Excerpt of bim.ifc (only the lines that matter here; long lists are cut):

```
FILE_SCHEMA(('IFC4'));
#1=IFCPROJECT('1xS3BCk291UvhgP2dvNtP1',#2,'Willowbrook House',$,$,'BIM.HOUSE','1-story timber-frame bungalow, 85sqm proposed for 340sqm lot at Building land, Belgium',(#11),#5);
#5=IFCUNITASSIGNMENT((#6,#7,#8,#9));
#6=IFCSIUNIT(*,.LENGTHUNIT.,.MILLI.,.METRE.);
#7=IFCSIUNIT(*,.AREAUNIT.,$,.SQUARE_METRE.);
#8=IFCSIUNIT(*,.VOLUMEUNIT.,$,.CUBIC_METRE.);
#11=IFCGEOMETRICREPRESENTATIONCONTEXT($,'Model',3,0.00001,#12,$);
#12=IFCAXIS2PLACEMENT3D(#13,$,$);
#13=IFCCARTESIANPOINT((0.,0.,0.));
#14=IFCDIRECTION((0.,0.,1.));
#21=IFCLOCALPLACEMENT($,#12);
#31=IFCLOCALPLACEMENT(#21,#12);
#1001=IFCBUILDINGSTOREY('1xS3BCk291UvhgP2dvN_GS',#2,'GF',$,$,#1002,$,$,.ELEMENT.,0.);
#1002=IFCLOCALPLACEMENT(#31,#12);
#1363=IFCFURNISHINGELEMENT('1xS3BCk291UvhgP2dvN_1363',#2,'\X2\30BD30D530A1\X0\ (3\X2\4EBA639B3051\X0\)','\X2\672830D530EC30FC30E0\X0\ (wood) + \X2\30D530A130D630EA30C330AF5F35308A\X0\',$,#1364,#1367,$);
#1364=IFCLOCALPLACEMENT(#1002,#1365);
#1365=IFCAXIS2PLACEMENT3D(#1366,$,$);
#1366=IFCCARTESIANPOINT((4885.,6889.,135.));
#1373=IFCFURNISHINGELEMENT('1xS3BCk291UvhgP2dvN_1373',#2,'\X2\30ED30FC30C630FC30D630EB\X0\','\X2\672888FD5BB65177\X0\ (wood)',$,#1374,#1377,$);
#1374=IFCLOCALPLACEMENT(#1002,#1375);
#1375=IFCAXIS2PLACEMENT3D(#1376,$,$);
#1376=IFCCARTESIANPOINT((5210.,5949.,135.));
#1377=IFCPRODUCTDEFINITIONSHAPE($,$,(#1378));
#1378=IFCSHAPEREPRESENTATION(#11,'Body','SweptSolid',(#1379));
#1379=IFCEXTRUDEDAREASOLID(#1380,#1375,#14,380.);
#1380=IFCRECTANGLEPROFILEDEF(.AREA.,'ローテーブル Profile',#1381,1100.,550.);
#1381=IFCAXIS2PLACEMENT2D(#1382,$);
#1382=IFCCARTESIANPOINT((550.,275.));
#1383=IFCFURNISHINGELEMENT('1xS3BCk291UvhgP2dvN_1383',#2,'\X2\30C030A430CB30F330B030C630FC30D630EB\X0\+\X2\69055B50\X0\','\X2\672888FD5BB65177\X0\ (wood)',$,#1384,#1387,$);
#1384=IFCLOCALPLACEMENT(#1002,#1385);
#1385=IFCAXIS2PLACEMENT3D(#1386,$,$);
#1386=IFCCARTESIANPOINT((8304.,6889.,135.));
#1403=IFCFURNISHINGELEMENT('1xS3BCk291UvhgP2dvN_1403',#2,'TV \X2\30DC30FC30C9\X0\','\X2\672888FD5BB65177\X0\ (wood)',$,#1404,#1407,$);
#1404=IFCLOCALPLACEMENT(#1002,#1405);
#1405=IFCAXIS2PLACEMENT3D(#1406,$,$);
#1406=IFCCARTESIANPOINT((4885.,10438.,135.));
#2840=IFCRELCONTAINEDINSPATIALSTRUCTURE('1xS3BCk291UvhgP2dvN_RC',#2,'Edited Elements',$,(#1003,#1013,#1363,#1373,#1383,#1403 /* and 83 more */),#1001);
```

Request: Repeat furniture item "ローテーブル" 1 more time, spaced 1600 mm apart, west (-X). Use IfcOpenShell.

```python
import numpy as np
import ifcopenshell
import ifcopenshell.api.geometry
import ifcopenshell.api.root
import ifcopenshell.util.element
import ifcopenshell.util.placement
import ifcopenshell.util.unit

model = ifcopenshell.open("bim.ifc")
unit_scale = ifcopenshell.util.unit.calculate_unit_scale(model)


def reuse_history(source, copy):
    """copy_class also copies each property set's owner history, people and application; keep the originals."""
    for rel in copy.IsDefinedBy:
        if rel.is_a("IfcRelDefinesByProperties") and (history := rel.RelatingPropertyDefinition.OwnerHistory):
            rel.RelatingPropertyDefinition.OwnerHistory = source.OwnerHistory
            ifcopenshell.util.element.remove_deep2(model, history)


source = model.by_guid("1xS3BCk291UvhgP2dvN_1373")
base = ifcopenshell.util.placement.get_local_placement(source.ObjectPlacement)
step = np.array([-1.0, 0.0, 0.0]) * 1.6 / unit_scale

for i in range(1, 2):
    copy = ifcopenshell.api.root.copy_class(model, product=source)
    copy.Representation = ifcopenshell.util.element.copy_deep(
        model, source.Representation, exclude=["IfcGeometricRepresentationContext", "IfcRepresentationMap"]
    )
    reuse_history(source, copy)
    matrix = base.copy()
    matrix[:3, 3] += i * step
    print("added at", matrix[:3, 3].round(3) + 0.0)
    ifcopenshell.api.geometry.edit_object_placement(model, product=copy, matrix=matrix, is_si=False)

model.write("bim-out.ifc")
```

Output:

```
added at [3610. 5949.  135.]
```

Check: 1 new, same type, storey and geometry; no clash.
